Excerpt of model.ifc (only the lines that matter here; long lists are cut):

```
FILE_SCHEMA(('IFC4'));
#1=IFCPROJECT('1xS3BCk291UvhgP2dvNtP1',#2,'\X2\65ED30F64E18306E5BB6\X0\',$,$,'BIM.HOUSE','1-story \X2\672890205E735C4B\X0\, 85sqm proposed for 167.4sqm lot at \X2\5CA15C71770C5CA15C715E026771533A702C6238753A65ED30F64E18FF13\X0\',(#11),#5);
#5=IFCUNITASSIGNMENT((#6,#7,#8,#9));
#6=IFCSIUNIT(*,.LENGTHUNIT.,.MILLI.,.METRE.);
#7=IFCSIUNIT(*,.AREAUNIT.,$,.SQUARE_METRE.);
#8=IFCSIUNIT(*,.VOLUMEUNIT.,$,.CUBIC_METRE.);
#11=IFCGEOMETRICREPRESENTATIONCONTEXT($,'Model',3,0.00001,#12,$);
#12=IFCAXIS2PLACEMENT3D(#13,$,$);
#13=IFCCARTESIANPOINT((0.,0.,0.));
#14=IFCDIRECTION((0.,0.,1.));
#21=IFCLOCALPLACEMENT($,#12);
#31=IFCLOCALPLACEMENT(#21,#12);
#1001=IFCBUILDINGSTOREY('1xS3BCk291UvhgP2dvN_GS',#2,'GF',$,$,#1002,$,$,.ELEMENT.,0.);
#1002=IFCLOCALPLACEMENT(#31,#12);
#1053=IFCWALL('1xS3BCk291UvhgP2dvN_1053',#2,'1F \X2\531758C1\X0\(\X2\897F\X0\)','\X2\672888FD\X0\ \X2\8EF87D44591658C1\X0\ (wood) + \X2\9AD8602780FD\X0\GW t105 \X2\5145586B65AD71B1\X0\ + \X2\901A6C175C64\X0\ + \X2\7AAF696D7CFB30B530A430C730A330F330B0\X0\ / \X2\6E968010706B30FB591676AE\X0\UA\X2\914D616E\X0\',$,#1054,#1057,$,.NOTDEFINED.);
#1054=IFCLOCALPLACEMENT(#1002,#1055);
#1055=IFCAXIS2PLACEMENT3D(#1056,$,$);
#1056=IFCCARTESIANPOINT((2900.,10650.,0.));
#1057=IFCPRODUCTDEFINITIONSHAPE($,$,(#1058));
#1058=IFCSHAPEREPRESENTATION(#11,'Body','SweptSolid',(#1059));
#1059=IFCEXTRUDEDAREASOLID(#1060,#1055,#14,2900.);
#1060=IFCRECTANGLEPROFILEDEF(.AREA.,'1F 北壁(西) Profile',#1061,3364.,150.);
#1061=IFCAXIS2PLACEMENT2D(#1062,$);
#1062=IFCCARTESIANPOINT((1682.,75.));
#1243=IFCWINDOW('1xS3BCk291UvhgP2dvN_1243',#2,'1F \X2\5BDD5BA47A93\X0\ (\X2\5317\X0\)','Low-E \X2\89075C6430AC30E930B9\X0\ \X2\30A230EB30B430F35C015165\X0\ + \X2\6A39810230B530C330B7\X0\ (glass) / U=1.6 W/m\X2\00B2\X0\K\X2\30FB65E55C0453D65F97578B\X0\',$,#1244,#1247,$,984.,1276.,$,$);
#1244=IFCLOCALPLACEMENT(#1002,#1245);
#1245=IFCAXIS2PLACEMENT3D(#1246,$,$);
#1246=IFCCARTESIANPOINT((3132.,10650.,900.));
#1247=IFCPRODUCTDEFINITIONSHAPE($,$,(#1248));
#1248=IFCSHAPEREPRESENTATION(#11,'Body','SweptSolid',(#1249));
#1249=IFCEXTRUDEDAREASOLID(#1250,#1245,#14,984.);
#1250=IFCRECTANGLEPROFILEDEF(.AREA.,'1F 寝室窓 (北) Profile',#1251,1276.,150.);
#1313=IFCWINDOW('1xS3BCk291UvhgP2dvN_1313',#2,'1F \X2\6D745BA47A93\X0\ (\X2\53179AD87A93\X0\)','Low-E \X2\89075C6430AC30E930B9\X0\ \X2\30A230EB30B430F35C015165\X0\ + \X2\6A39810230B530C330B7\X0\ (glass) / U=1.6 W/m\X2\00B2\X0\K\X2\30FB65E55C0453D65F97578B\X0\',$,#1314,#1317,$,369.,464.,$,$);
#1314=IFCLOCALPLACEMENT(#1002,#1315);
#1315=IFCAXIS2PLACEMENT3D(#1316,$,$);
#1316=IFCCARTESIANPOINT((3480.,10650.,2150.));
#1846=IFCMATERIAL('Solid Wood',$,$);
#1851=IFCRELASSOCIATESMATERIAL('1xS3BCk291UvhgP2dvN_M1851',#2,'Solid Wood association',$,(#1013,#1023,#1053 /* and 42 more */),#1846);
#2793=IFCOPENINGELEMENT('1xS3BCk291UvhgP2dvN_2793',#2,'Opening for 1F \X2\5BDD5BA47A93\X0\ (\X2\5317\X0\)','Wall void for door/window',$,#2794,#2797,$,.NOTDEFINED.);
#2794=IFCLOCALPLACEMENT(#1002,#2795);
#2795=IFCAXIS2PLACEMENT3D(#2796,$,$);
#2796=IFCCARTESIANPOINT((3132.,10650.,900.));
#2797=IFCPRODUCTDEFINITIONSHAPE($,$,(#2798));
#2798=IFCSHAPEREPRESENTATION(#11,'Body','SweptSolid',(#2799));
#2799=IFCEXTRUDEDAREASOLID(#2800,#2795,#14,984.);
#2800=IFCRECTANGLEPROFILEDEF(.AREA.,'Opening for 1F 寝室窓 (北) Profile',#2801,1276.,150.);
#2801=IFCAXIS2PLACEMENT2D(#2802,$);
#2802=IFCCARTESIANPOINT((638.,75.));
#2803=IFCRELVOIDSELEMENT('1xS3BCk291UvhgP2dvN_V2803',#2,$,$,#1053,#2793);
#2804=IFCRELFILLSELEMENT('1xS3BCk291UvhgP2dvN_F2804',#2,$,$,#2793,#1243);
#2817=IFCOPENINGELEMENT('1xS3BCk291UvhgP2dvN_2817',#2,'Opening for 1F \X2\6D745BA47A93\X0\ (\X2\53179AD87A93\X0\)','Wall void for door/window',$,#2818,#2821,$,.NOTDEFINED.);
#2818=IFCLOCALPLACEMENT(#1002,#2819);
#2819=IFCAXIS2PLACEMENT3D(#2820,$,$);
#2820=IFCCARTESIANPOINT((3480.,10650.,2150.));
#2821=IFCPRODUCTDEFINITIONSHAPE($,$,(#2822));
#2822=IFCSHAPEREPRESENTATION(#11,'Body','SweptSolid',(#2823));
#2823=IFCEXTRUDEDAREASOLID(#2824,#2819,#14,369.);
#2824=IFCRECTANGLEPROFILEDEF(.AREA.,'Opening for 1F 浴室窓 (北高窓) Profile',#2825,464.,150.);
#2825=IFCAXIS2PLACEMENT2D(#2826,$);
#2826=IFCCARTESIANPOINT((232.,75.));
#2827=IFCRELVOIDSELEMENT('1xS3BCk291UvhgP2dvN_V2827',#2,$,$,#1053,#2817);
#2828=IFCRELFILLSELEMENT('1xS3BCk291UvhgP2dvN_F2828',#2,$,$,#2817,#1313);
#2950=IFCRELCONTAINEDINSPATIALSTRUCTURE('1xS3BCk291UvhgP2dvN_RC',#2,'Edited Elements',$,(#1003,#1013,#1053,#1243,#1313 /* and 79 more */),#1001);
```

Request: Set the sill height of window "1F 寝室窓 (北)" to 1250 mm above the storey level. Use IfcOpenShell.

```python
import numpy as np
import ifcopenshell
import ifcopenshell.api.geometry
import ifcopenshell.geom
import ifcopenshell.util.element
import ifcopenshell.util.placement
import ifcopenshell.util.shape
import ifcopenshell.util.unit

model = ifcopenshell.open("model.ifc")
unit_scale = ifcopenshell.util.unit.calculate_unit_scale(model)

window = model.by_guid("1xS3BCk291UvhgP2dvN_1243")
opening = window.FillsVoids[0].RelatingOpeningElement
storey = ifcopenshell.util.element.get_container(window, ifc_class="IfcBuildingStorey")
level = ifcopenshell.util.placement.get_local_placement(storey.ObjectPlacement)[2, 3]

# The opening's origin need not be at the sill, so measure its lowest point.
shape = ifcopenshell.geom.create_shape(ifcopenshell.geom.settings(), opening)
bottom = ifcopenshell.util.shape.get_shape_bottom_elevation(shape, shape.geometry) / unit_scale
dz = level + 1.25 / unit_scale - bottom

shift = np.array([0.0, 0.0, dz])
# The window is not placed relative to its opening, so move both.
for product in (opening, window):
    matrix = ifcopenshell.util.placement.get_local_placement(product.ObjectPlacement)
    matrix[:3, 3] += shift
    ifcopenshell.api.geometry.edit_object_placement(model, product=product, matrix=matrix, is_si=False)

print(f"moved by {dz * unit_scale:+.3f} m")

model.write("model-out.ifc")
```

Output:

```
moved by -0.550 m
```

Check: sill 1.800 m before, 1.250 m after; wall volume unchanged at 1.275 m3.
